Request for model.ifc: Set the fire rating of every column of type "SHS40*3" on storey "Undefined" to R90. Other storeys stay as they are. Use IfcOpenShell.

First a look at what the model holds.

```python
import ifcopenshell
import ifcopenshell.util.element

model = ifcopenshell.open("model.ifc")
print(model.schema)
storey = next(s for s in model.by_type("IfcBuildingStorey") if s.Name == "Undefined")
columns = [e for e in ifcopenshell.util.element.get_decomposition(storey) if e.is_a("IfcColumn")]
seen = {}
for e in columns:
    element_type = ifcopenshell.util.element.get_type(e)
    key = (element_type.Name if element_type != e and element_type else None, ifcopenshell.util.element.get_pset(e, "Pset_ColumnCommon", "FireRating"))
    seen[key] = seen.get(key, 0) + 1
for (name, value), count in sorted(seen.items(), key=str):
    print(count, "x", name, "|", value)
```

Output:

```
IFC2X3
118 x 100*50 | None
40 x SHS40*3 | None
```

```python
import ifcopenshell
import ifcopenshell.api.pset
import ifcopenshell.util.element

model = ifcopenshell.open("model.ifc")

storey = next(s for s in model.by_type("IfcBuildingStorey") if s.Name == "Undefined")
columns = [e for e in ifcopenshell.util.element.get_decomposition(storey) if e.is_a("IfcColumn")]

count = 0
for e in columns:
    element_type = ifcopenshell.util.element.get_type(e)
    if element_type in (None, e) or element_type.Name != "SHS40*3":
        continue
    # add_pset returns the element's existing set when there is one.
    pset = ifcopenshell.api.pset.add_pset(model, product=e, name="Pset_ColumnCommon")
    ifcopenshell.api.pset.edit_pset(model, pset=pset, properties={"FireRating": "R90"})
    count += 1

print(count, "columns updated")

model.write("model_v2.ifc")
```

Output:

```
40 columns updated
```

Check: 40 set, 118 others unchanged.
